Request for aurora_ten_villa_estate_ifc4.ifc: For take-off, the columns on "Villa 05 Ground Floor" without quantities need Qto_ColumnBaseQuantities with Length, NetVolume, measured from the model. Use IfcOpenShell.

First a look at what the model holds.

```python
import ifcopenshell
import ifcopenshell.util.element
import ifcopenshell.util.unit

model = ifcopenshell.open("aurora_ten_villa_estate_ifc4.ifc")
print(model.schema)
for unit_type in ("LENGTHUNIT", "AREAUNIT", "VOLUMEUNIT"):
    print(unit_type, ifcopenshell.util.unit.calculate_unit_scale(model, unit_type))
storey = next(s for s in model.by_type("IfcBuildingStorey") if s.Name == "Villa 05 Ground Floor")
columns = [e for e in ifcopenshell.util.element.get_decomposition(storey) if e.is_a("IfcColumn")]
for e in sorted(columns, key=lambda e: e.id()):
    print(e.id(), e.is_a(), e.Name, list(ifcopenshell.util.element.get_psets(e, qtos_only=True)), sep=" | ")
```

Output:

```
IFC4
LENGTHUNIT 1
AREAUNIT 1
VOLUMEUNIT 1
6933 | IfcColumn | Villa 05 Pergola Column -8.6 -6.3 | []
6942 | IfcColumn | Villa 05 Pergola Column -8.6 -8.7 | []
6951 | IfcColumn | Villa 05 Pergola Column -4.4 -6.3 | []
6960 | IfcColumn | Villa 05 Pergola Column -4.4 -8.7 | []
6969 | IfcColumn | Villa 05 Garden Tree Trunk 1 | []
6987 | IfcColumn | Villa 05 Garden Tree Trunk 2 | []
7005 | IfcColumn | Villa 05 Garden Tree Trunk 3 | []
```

```python
import ifcopenshell
import ifcopenshell.api.pset
import ifcopenshell.geom
import ifcopenshell.util.element
import ifcopenshell.util.shape
import ifcopenshell.util.unit

model = ifcopenshell.open("aurora_ten_villa_estate_ifc4.ifc")
unit_scale = ifcopenshell.util.unit.calculate_unit_scale(model)
volume_scale = ifcopenshell.util.unit.calculate_unit_scale(model, "VOLUMEUNIT")
settings = ifcopenshell.geom.settings()

storey = next(s for s in model.by_type("IfcBuildingStorey") if s.Name == "Villa 05 Ground Floor")
columns = [e for e in ifcopenshell.util.element.get_decomposition(storey) if e.is_a("IfcColumn")]

for e in sorted(columns, key=lambda e: e.id()):
    if ifcopenshell.util.element.get_psets(e, qtos_only=True, should_inherit=False):
        continue
    # Geometry comes back in metres, in the element's own axes.
    shape = ifcopenshell.geom.create_shape(settings, e)
    values = {
        "Length": ifcopenshell.util.shape.get_z(shape.geometry) / unit_scale,
        "NetVolume": ifcopenshell.util.shape.get_volume(shape.geometry) / volume_scale,
    }
    qto = ifcopenshell.api.pset.add_qto(model, product=e, name="Qto_ColumnBaseQuantities")
    ifcopenshell.api.pset.edit_qto(model, qto=qto, properties=values)
    print(e.id(), {k: round(v, 3) for k, v in values.items()})

model.write("aurora_ten_villa_estate_ifc4_updated.ifc")
```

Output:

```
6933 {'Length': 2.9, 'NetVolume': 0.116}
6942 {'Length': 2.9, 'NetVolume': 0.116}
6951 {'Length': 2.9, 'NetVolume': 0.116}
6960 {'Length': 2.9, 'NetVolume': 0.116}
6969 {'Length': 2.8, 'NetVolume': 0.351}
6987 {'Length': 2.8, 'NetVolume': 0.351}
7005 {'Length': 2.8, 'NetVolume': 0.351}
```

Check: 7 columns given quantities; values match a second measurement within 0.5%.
